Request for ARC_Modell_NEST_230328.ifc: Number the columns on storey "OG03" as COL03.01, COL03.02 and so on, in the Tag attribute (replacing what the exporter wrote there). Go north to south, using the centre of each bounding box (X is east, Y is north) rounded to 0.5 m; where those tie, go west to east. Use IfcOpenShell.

First a look at what the model holds.

```python
import ifcopenshell
import ifcopenshell.util.element
import ifcopenshell.util.placement

model = ifcopenshell.open("ARC_Modell_NEST_230328.ifc")
print(model.schema)
storey = next(s for s in model.by_type("IfcBuildingStorey") if s.Name == "OG03")
columns = [e for e in ifcopenshell.util.element.get_decomposition(storey) if e.is_a("IfcColumn")]
for e in sorted(columns, key=lambda e: e.id()):
    origin = ifcopenshell.util.placement.get_local_placement(e.ObjectPlacement)[:3, 3]
    print(e.id(), e.Tag, e.Name, origin.round(2) + 0.0, sep=" | ")
```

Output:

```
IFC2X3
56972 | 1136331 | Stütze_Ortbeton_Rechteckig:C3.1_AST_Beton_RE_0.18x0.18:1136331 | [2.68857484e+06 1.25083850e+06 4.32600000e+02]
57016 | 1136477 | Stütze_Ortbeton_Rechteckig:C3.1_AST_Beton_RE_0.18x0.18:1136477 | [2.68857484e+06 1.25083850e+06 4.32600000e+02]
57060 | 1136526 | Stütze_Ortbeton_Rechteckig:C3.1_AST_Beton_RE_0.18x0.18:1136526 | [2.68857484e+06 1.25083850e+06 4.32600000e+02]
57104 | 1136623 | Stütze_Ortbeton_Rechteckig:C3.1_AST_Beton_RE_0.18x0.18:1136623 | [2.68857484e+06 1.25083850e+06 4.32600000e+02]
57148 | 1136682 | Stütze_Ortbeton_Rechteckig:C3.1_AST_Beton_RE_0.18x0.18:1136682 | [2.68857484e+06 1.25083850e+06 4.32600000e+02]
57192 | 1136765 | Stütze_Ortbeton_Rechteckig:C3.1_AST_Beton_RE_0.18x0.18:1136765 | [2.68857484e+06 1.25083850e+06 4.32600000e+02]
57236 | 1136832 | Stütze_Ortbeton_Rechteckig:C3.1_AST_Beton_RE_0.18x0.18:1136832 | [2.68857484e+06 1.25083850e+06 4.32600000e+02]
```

```python
import ifcopenshell
import ifcopenshell.geom
import ifcopenshell.util.element
import ifcopenshell.util.shape

model = ifcopenshell.open("ARC_Modell_NEST_230328.ifc")
settings = ifcopenshell.geom.settings()
settings.set("use-world-coords", True)


def centre(element):
    shape = ifcopenshell.geom.create_shape(settings, element)
    return ifcopenshell.util.shape.get_bbox_centroid(shape.geometry)


storey = next(s for s in model.by_type("IfcBuildingStorey") if s.Name == "OG03")
columns = [e for e in ifcopenshell.util.element.get_decomposition(storey) if e.is_a("IfcColumn")]

# Insertion points can sit at a corner or the storey origin, so sort by the geometry (in metres).
centres = {e: centre(e) for e in columns}
columns.sort(key=lambda e: (-round(centres[e][1] / 0.5), centres[e][0]))

for i, e in enumerate(columns, start=1):
    number = f"COL03.{i:02d}"
    e.Tag = number
    print(e.id(), number)

model.write("ARC_Modell_NEST_230328_updated.ifc")
```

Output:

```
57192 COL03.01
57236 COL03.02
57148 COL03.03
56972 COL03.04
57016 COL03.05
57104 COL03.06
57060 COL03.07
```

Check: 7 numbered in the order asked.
